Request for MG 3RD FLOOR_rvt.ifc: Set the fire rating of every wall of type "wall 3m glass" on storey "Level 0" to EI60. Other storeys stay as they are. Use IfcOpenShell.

First a look at what the model holds.

```python
import ifcopenshell
import ifcopenshell.util.element

model = ifcopenshell.open("MG 3RD FLOOR_rvt.ifc")
print(model.schema)
storey = next(s for s in model.by_type("IfcBuildingStorey") if s.Name == "Level 0")
walls = [e for e in ifcopenshell.util.element.get_decomposition(storey) if e.is_a("IfcWall")]
seen = {}
for e in walls:
    element_type = ifcopenshell.util.element.get_type(e)
    key = (element_type.Name if element_type != e and element_type else None, ifcopenshell.util.element.get_pset(e, "Pset_WallCommon", "FireRating"))
    seen[key] = seen.get(key, 0) + 1
for (name, value), count in sorted(seen.items(), key=str):
    print(count, "x", name, "|", value)
```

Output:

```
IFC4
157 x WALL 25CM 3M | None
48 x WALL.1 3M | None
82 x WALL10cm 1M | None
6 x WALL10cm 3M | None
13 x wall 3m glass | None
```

```python
import ifcopenshell
import ifcopenshell.api.pset
import ifcopenshell.util.element

model = ifcopenshell.open("MG 3RD FLOOR_rvt.ifc")

storey = next(s for s in model.by_type("IfcBuildingStorey") if s.Name == "Level 0")
walls = [e for e in ifcopenshell.util.element.get_decomposition(storey) if e.is_a("IfcWall")]

count = 0
for e in walls:
    element_type = ifcopenshell.util.element.get_type(e)
    if element_type in (None, e) or element_type.Name != "wall 3m glass":
        continue
    # add_pset returns the element's existing set when there is one.
    pset = ifcopenshell.api.pset.add_pset(model, product=e, name="Pset_WallCommon")
    ifcopenshell.api.pset.edit_pset(model, pset=pset, properties={"FireRating": "EI60"})
    count += 1

print(count, "walls updated")

model.write("MG 3RD FLOOR_rvt_v2.ifc")
```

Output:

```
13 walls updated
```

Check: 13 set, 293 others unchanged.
